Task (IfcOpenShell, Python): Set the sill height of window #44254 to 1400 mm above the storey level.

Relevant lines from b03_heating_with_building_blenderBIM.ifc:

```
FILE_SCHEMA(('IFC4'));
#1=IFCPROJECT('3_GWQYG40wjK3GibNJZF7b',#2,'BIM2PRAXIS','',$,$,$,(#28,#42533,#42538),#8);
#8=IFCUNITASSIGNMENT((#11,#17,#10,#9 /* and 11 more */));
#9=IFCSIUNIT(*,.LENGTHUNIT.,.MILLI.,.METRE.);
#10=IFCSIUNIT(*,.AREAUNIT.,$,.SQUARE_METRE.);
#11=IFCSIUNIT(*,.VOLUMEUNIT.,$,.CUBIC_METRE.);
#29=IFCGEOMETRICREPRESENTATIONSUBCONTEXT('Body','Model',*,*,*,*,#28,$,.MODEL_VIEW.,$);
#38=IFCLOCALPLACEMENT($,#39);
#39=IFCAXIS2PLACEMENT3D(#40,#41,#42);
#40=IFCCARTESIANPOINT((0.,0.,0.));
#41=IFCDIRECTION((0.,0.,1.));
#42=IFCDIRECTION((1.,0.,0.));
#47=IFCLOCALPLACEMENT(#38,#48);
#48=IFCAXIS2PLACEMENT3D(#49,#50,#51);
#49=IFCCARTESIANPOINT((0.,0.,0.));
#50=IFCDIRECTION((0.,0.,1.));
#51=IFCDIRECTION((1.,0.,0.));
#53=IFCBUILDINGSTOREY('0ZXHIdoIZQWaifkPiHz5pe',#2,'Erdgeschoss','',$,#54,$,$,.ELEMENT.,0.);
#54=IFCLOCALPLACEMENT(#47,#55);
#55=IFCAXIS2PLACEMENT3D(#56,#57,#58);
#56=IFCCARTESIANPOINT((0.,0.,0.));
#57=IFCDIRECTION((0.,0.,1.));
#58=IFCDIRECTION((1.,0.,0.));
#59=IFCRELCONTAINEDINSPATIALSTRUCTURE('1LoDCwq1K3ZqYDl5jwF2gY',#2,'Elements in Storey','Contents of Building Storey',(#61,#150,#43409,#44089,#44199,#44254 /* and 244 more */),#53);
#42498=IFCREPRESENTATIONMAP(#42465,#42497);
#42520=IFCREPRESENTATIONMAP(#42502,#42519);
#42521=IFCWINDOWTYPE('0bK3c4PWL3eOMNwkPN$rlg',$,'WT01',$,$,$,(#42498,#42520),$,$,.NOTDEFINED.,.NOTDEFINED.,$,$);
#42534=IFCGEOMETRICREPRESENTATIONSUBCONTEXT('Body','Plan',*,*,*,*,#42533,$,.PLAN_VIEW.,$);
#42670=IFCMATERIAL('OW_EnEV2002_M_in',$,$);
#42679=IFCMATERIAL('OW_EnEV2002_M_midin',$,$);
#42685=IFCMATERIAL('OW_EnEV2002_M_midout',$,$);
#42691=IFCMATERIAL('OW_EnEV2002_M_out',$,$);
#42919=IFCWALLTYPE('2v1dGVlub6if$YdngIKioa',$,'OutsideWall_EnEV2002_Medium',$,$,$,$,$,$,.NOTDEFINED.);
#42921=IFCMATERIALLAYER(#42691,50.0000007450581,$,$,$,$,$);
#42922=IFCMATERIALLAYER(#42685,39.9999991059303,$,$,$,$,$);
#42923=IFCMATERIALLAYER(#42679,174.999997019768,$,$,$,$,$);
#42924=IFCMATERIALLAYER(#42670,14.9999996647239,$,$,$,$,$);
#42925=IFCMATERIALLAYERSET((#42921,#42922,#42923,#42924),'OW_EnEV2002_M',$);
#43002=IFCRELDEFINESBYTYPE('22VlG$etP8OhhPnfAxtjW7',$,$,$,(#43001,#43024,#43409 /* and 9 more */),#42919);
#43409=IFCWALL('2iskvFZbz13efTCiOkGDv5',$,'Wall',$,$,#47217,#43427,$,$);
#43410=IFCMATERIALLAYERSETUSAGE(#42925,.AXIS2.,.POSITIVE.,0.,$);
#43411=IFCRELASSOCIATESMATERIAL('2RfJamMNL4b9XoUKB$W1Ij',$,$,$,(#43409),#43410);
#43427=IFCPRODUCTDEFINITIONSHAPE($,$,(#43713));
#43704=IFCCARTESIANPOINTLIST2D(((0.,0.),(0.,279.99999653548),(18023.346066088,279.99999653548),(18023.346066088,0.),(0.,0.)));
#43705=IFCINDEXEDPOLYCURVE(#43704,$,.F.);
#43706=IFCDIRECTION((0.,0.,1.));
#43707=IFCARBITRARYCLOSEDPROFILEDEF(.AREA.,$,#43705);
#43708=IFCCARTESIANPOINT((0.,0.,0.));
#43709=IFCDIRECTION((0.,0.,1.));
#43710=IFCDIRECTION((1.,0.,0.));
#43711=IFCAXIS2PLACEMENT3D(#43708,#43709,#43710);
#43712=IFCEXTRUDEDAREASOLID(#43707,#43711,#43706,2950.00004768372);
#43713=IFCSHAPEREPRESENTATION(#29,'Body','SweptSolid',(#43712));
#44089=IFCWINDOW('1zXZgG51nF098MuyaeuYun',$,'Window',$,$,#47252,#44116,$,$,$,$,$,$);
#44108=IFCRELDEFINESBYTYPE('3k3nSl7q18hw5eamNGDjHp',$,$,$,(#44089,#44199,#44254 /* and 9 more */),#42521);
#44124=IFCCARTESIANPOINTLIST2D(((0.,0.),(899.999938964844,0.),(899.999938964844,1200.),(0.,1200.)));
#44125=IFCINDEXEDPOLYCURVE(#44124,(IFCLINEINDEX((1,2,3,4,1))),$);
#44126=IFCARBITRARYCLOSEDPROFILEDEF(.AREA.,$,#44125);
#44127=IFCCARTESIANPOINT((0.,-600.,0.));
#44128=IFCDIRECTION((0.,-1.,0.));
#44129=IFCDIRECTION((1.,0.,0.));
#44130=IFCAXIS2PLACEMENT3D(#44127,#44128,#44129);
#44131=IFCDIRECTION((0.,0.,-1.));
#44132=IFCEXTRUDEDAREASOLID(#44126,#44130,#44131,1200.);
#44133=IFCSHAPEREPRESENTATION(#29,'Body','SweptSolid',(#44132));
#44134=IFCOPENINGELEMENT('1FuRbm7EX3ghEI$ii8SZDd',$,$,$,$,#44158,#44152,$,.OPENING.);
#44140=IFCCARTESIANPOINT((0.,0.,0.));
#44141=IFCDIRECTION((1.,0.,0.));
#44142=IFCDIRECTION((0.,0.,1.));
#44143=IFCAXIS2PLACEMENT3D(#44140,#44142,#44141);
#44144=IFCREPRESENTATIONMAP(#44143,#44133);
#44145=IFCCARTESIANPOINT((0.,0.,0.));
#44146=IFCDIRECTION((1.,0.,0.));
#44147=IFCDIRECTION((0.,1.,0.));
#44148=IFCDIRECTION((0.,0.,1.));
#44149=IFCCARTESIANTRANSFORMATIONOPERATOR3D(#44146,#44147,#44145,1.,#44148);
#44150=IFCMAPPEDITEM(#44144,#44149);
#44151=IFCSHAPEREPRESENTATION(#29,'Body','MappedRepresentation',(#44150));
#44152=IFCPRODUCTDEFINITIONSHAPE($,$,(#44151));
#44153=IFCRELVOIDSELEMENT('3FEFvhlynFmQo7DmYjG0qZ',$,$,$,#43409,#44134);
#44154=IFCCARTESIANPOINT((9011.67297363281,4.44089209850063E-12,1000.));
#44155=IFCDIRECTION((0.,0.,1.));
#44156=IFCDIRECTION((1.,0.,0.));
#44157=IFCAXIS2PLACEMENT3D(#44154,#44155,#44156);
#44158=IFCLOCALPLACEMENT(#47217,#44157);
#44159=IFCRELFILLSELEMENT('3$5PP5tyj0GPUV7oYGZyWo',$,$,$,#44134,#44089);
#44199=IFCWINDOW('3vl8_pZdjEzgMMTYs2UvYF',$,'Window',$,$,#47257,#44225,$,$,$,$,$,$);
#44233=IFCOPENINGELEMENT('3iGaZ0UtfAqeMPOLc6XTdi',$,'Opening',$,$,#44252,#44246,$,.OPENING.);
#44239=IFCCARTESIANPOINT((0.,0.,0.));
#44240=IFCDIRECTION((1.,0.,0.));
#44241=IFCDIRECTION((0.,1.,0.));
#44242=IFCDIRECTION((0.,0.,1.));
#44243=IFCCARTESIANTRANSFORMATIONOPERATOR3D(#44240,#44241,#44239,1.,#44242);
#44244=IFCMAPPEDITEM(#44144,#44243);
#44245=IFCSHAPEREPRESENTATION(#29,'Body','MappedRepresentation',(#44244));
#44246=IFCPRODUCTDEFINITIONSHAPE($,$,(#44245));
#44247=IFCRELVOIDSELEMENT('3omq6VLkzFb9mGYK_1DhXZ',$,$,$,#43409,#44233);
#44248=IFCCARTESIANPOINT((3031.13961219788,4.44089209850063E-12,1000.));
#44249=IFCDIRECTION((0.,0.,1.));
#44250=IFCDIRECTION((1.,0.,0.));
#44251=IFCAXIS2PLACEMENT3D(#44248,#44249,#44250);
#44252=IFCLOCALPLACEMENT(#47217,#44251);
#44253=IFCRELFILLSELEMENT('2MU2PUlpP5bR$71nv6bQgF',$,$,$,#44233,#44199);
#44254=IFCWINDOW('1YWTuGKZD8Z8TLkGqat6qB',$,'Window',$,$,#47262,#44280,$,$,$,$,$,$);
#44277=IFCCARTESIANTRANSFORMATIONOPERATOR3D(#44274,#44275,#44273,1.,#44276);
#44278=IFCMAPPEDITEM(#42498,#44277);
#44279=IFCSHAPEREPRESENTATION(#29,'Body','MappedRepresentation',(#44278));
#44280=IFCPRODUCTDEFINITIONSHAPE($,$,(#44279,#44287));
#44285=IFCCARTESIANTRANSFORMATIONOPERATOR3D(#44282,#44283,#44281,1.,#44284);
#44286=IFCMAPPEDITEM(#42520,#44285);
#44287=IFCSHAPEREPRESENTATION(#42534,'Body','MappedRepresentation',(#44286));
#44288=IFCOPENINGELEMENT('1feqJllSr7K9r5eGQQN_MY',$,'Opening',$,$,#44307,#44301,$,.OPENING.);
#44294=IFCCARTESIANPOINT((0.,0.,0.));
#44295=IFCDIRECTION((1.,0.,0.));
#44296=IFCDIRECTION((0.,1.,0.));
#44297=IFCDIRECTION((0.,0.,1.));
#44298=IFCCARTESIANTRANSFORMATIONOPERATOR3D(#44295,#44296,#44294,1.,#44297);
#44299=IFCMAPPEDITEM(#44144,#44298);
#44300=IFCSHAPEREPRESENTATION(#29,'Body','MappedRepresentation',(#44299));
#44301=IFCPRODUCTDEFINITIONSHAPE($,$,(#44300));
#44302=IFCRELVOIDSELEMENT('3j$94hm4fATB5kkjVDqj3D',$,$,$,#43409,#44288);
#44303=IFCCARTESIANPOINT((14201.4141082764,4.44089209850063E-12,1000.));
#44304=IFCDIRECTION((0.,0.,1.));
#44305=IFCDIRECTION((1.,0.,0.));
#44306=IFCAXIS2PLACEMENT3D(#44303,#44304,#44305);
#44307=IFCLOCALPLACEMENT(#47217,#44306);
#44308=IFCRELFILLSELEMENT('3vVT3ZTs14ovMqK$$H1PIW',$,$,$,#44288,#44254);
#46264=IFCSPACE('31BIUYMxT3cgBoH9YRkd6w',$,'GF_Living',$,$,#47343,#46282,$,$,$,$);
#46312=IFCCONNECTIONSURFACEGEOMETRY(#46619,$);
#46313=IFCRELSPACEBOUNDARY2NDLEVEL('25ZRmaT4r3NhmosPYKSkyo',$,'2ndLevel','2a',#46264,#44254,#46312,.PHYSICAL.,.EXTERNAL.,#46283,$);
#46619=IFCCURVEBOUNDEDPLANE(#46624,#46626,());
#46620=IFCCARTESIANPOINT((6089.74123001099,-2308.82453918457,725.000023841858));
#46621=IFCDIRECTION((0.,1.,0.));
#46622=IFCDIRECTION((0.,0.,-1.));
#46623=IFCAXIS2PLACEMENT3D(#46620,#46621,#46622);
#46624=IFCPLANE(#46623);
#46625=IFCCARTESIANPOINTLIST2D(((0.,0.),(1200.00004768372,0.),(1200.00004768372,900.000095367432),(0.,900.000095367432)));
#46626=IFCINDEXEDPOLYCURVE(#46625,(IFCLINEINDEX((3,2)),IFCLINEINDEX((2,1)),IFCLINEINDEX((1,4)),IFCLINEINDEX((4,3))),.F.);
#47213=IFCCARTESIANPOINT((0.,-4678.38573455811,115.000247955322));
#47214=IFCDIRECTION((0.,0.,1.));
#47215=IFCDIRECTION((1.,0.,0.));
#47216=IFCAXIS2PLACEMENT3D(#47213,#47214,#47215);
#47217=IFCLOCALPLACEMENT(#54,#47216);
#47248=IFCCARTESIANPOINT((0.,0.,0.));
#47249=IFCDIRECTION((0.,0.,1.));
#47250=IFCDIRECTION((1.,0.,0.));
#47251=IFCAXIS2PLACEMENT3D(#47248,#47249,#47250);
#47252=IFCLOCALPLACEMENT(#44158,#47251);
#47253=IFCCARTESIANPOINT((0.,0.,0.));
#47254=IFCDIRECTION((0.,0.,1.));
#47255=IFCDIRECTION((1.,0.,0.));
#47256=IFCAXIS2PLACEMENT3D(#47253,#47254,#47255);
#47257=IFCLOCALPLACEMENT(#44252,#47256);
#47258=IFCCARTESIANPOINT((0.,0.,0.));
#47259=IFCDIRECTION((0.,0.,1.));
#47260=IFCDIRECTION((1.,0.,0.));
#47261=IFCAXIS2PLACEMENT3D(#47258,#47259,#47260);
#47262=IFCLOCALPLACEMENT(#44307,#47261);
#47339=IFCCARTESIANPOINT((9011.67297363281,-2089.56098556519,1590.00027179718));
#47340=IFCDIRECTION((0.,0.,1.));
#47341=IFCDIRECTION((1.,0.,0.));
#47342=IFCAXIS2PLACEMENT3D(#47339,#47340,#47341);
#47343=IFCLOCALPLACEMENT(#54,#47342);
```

```python
import numpy as np
import ifcopenshell
import ifcopenshell.api.geometry
import ifcopenshell.geom
import ifcopenshell.util.element
import ifcopenshell.util.placement
import ifcopenshell.util.shape
import ifcopenshell.util.unit

model = ifcopenshell.open("b03_heating_with_building_blenderBIM.ifc")
unit_scale = ifcopenshell.util.unit.calculate_unit_scale(model)

window = model.by_guid("1YWTuGKZD8Z8TLkGqat6qB")
opening = window.FillsVoids[0].RelatingOpeningElement
storey = ifcopenshell.util.element.get_container(window, ifc_class="IfcBuildingStorey")
level = ifcopenshell.util.placement.get_local_placement(storey.ObjectPlacement)[2, 3]

# The opening's origin need not be at the sill, so measure its lowest point.
shape = ifcopenshell.geom.create_shape(ifcopenshell.geom.settings(), opening)
bottom = ifcopenshell.util.shape.get_shape_bottom_elevation(shape, shape.geometry) / unit_scale
dz = level + 1.4 / unit_scale - bottom

shift = np.array([0.0, 0.0, dz])
# The window is placed relative to its opening, so it follows when the opening moves.
matrix = ifcopenshell.util.placement.get_local_placement(opening.ObjectPlacement)
matrix[:3, 3] += shift
ifcopenshell.api.geometry.edit_object_placement(
    model, product=opening, matrix=matrix, is_si=False, should_transform_children=True
)

# Space boundary surfaces are stored in each space's coordinates; move them too.
for rel in window.ProvidesBoundaries:
    if not rel.ConnectionGeometry:
        continue
    surface = rel.ConnectionGeometry.SurfaceOnRelatingElement.BasisSurface
    space_matrix = ifcopenshell.util.placement.get_local_placement(rel.RelatingSpace.ObjectPlacement)
    point = np.array(surface.Position.Location.Coordinates) + space_matrix[:3, :3].T @ shift
    surface.Position = model.createIfcAxis2Placement3D(
        model.createIfcCartesianPoint(point.tolist()), surface.Position.Axis, surface.Position.RefDirection
    )

print(f"moved by {dz * unit_scale:+.3f} m")

model.write("b03_heating_with_building_blenderBIM_updated.ifc")
```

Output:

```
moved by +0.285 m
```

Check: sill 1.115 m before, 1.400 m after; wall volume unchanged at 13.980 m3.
